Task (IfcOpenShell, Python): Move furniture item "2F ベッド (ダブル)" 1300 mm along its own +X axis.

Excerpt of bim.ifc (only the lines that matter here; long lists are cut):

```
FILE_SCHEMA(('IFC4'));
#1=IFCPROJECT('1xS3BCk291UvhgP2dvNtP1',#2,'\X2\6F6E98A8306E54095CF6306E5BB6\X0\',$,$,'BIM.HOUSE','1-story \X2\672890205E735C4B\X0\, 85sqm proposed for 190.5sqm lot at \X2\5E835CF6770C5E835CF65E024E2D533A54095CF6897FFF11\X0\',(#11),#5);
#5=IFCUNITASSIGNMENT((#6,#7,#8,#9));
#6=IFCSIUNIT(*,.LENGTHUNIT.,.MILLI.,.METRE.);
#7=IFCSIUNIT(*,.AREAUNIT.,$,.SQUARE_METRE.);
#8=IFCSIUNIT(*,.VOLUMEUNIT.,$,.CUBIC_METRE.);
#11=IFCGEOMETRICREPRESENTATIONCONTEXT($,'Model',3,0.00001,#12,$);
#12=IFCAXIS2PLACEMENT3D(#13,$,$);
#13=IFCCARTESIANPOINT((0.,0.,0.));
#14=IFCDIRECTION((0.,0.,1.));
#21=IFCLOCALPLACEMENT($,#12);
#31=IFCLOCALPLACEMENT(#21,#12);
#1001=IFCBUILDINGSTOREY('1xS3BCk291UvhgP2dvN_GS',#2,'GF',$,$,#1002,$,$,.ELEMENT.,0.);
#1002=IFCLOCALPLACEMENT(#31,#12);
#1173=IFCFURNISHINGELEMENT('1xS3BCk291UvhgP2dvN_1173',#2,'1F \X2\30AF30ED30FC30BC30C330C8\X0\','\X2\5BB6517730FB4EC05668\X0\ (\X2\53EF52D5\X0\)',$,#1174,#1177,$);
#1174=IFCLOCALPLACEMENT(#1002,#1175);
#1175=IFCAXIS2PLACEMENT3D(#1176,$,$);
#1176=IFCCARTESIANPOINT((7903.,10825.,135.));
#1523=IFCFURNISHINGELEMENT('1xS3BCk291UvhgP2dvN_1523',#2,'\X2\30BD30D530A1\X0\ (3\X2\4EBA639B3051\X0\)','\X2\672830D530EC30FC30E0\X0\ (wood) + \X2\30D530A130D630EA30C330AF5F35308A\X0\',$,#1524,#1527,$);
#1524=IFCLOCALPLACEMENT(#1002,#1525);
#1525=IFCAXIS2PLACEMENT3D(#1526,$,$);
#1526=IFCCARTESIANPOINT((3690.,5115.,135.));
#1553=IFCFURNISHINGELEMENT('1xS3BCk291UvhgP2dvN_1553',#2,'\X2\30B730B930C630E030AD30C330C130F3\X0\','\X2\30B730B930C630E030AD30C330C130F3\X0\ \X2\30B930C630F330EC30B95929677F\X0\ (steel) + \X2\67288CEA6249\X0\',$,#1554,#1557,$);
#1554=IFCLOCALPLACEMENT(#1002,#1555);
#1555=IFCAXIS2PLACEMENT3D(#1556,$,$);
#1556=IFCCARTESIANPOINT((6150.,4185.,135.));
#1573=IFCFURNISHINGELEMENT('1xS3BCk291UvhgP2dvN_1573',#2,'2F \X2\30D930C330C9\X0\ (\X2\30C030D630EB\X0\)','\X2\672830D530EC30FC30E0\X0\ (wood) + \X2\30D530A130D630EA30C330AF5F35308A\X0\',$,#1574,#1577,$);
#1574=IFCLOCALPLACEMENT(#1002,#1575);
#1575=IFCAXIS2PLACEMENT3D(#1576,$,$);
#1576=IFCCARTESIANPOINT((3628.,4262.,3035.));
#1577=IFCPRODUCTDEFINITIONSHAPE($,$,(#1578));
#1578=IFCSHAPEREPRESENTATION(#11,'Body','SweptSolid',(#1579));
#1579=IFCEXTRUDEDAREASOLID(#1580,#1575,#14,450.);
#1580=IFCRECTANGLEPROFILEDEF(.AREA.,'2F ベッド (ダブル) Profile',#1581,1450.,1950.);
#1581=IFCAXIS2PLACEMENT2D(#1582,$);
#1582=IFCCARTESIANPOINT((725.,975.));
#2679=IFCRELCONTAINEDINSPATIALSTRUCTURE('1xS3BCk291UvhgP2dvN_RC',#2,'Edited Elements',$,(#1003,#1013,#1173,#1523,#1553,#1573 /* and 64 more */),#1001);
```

```python
import ifcopenshell
import ifcopenshell.api.geometry
import ifcopenshell.util.placement
import ifcopenshell.util.unit

model = ifcopenshell.open("bim.ifc")
unit_scale = ifcopenshell.util.unit.calculate_unit_scale(model)

item = model.by_guid("1xS3BCk291UvhgP2dvN_1573")
matrix = ifcopenshell.util.placement.get_local_placement(item.ObjectPlacement)
matrix[:3, 3] += matrix[:3, 0] * 1.3 / unit_scale
ifcopenshell.api.geometry.edit_object_placement(model, product=item, matrix=matrix, is_si=False)

print(ifcopenshell.util.placement.get_local_placement(item.ObjectPlacement).round(3) + 0.0)

model.write("bim_edited.ifc")
```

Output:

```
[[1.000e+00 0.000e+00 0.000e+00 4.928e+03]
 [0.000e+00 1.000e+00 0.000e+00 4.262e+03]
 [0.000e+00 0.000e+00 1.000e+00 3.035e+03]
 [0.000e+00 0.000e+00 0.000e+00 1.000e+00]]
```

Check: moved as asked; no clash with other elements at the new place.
